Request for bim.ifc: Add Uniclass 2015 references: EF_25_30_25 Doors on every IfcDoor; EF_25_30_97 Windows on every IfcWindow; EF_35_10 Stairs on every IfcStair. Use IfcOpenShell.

First a look at what the model holds.

```python
import ifcopenshell

model = ifcopenshell.open("bim.ifc")
print(model.schema)
print("classifications:", [c.Name for c in model.by_type("IfcClassification")])
for ifc_class in ("IfcDoor", "IfcRoof", "IfcStair", "IfcWall", "IfcWindow"):
    print(ifc_class, len(model.by_type(ifc_class)))
```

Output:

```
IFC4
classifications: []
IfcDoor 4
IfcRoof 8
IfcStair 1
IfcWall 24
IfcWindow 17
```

```python
import ifcopenshell
import ifcopenshell.api.classification

model = ifcopenshell.open("bim.ifc")

system = ifcopenshell.api.classification.add_classification(model, classification="Uniclass 2015")

codes = {
    "IfcDoor": ("EF_25_30_25", "Doors"),
    "IfcWindow": ("EF_25_30_97", "Windows"),
    "IfcStair": ("EF_35_10", "Stairs"),
}
for ifc_class, (code, name) in codes.items():
    products = model.by_type(ifc_class)
    ifcopenshell.api.classification.add_reference(
        model, products=products, classification=system, identification=code, name=name
    )
    print(code, len(products))

model.write("bim_rev.ifc")
```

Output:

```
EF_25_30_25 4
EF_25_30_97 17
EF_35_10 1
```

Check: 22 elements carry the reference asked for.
